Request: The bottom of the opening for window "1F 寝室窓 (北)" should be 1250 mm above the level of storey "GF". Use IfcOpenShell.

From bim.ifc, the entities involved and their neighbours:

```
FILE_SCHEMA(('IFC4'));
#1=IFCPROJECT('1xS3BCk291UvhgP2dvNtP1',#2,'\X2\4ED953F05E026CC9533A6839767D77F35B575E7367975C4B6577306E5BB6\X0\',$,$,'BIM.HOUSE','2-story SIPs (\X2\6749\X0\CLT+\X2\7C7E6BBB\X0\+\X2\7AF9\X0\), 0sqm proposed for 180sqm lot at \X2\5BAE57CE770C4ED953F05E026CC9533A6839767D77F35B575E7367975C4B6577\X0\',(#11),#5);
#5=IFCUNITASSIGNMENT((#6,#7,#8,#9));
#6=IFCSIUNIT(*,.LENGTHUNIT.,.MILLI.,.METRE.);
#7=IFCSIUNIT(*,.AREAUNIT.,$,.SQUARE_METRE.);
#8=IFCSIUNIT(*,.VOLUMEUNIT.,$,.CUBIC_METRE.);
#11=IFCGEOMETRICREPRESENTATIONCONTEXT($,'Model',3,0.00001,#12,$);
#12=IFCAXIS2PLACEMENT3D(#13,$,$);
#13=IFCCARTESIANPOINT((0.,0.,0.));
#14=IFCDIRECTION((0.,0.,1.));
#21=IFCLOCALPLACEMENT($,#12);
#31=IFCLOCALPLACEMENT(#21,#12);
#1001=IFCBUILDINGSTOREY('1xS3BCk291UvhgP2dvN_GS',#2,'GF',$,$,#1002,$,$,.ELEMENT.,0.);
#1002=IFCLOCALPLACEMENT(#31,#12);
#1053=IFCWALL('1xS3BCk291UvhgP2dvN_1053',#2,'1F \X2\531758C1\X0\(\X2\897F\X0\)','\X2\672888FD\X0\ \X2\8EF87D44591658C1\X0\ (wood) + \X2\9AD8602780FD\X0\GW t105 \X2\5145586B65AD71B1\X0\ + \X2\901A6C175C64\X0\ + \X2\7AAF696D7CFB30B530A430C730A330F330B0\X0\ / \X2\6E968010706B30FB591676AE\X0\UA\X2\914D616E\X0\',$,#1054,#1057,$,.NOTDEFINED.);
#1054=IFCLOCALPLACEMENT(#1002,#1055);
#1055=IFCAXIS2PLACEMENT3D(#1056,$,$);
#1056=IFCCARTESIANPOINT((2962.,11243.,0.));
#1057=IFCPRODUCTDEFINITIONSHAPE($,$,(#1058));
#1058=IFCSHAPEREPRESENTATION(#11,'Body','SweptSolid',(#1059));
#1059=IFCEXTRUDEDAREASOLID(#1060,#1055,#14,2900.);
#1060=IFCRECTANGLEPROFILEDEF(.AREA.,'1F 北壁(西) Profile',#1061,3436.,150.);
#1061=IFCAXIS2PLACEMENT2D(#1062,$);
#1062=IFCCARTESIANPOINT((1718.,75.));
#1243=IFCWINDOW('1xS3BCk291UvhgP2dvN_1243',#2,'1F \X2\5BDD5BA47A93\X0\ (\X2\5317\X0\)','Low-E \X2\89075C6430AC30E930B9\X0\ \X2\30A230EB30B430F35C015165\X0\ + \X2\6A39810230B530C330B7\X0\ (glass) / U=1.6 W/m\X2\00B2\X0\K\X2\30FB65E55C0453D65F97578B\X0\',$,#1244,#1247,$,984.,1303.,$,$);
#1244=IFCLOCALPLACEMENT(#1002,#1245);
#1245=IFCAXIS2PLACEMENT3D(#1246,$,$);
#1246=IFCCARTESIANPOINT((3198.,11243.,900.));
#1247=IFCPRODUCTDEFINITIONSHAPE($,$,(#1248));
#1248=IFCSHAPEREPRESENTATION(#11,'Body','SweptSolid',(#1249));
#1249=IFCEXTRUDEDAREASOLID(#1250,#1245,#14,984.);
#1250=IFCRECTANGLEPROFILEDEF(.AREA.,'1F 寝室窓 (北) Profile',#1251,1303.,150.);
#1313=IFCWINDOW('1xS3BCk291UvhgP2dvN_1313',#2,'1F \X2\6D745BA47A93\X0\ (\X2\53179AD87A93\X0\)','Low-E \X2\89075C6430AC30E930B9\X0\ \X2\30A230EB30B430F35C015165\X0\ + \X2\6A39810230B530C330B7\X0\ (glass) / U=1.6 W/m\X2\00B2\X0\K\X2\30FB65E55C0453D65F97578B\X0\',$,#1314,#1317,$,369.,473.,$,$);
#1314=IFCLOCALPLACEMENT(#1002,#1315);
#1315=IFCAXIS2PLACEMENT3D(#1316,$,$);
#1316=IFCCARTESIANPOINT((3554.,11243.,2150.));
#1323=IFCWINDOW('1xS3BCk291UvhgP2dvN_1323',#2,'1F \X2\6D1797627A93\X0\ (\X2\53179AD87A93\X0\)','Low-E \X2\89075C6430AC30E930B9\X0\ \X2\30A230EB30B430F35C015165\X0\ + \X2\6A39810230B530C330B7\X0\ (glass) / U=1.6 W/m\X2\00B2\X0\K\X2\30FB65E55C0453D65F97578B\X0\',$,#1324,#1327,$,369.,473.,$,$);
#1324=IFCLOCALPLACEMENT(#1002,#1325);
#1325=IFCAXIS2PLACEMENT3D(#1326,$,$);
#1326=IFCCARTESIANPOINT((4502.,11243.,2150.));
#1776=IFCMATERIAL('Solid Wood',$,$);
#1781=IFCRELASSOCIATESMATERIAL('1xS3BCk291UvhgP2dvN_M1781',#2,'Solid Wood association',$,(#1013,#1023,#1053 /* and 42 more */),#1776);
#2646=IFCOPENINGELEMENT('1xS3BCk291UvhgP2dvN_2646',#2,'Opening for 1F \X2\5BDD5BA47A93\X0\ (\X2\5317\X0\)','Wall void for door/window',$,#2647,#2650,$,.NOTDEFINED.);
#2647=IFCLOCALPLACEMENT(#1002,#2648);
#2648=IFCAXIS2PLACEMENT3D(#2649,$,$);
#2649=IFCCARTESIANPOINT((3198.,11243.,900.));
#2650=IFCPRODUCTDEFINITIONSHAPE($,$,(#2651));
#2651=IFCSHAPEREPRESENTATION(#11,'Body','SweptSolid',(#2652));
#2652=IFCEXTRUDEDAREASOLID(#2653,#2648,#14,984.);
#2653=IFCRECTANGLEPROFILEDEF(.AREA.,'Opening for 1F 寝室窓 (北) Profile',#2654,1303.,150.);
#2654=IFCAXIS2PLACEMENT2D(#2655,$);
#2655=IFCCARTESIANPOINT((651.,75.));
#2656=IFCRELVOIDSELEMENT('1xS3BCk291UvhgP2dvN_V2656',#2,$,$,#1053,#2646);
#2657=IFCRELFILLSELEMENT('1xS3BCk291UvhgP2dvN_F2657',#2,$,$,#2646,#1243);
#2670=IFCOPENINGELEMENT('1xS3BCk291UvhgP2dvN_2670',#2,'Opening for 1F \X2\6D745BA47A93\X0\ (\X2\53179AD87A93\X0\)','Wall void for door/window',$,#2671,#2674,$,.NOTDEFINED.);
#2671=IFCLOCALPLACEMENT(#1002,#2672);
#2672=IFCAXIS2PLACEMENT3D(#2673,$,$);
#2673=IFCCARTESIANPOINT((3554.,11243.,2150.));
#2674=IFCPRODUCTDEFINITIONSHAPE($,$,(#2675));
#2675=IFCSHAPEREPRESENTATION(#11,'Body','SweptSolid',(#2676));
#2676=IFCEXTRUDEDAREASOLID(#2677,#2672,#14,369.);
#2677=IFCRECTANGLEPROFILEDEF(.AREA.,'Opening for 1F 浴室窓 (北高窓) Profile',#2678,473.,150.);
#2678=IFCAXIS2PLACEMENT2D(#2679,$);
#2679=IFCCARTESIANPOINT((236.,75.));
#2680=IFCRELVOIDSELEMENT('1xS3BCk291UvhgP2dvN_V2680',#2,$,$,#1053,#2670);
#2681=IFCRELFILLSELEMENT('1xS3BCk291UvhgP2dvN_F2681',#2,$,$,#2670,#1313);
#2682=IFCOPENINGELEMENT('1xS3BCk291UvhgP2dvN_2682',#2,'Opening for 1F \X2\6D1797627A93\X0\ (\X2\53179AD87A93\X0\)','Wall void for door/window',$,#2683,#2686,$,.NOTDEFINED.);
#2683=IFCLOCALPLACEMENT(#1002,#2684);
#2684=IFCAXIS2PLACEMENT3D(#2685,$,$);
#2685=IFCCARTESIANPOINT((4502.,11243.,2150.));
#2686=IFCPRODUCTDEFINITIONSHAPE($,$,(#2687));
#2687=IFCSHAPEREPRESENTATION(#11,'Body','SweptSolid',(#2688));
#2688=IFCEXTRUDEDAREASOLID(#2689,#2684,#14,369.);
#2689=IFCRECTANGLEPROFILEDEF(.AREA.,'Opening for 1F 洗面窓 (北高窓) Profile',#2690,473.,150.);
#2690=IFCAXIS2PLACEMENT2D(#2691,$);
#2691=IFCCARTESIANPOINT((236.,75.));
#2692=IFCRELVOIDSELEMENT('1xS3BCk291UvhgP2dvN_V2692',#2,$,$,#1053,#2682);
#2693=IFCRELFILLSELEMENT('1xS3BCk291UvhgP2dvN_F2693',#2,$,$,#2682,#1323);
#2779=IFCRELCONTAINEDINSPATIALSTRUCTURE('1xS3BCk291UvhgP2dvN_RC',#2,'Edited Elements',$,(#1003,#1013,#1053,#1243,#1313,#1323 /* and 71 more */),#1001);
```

```python
import numpy as np
import ifcopenshell
import ifcopenshell.api.geometry
import ifcopenshell.geom
import ifcopenshell.util.element
import ifcopenshell.util.placement
import ifcopenshell.util.shape
import ifcopenshell.util.unit

model = ifcopenshell.open("bim.ifc")
unit_scale = ifcopenshell.util.unit.calculate_unit_scale(model)

window = model.by_id(1243)
opening = window.FillsVoids[0].RelatingOpeningElement
storey = ifcopenshell.util.element.get_container(window, ifc_class="IfcBuildingStorey")
level = ifcopenshell.util.placement.get_local_placement(storey.ObjectPlacement)[2, 3]

# The opening's origin need not be at the sill, so measure its lowest point.
shape = ifcopenshell.geom.create_shape(ifcopenshell.geom.settings(), opening)
bottom = ifcopenshell.util.shape.get_shape_bottom_elevation(shape, shape.geometry) / unit_scale
dz = level + 1.25 / unit_scale - bottom

shift = np.array([0.0, 0.0, dz])
# The window is not placed relative to its opening, so move both.
for product in (opening, window):
    matrix = ifcopenshell.util.placement.get_local_placement(product.ObjectPlacement)
    matrix[:3, 3] += shift
    ifcopenshell.api.geometry.edit_object_placement(model, product=product, matrix=matrix, is_si=False)

print(f"moved by {dz * unit_scale:+.3f} m")

model.write("bim_edited.ifc")
```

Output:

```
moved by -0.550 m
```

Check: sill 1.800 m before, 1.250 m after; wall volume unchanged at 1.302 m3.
